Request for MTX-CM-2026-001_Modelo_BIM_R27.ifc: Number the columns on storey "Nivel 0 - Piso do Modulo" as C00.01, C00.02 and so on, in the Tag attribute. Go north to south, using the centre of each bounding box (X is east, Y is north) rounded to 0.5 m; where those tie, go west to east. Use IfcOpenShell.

First a look at what the model holds.

```python
import ifcopenshell
import ifcopenshell.util.element
import ifcopenshell.util.placement

model = ifcopenshell.open("MTX-CM-2026-001_Modelo_BIM_R27.ifc")
print(model.schema)
storey = next(s for s in model.by_type("IfcBuildingStorey") if s.Name == "Nivel 0 - Piso do Modulo")
columns = [e for e in ifcopenshell.util.element.get_decomposition(storey) if e.is_a("IfcColumn")]
for e in sorted(columns, key=lambda e: e.id()):
    origin = ifcopenshell.util.placement.get_local_placement(e.ObjectPlacement)[:3, 3]
    print(e.id(), e.Tag, e.Name, origin.round(2) + 0.0, sep=" | ")
```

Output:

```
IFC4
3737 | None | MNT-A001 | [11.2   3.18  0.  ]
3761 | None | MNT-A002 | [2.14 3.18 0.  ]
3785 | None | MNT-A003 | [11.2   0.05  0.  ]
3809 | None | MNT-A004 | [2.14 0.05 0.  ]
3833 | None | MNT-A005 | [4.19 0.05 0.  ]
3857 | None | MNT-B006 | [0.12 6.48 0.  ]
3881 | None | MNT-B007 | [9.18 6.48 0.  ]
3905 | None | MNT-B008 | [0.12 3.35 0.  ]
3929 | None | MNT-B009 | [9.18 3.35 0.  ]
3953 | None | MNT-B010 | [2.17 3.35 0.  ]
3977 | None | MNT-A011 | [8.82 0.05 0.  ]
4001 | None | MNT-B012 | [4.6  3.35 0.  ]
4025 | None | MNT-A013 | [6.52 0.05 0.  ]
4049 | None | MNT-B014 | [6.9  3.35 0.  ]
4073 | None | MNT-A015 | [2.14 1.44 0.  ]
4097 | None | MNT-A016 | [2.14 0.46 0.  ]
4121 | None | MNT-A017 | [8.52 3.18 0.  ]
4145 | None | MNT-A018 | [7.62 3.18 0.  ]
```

```python
import ifcopenshell
import ifcopenshell.geom
import ifcopenshell.util.element
import ifcopenshell.util.shape

model = ifcopenshell.open("MTX-CM-2026-001_Modelo_BIM_R27.ifc")
settings = ifcopenshell.geom.settings()
settings.set("use-world-coords", True)


def centre(element):
    shape = ifcopenshell.geom.create_shape(settings, element)
    return ifcopenshell.util.shape.get_bbox_centroid(shape.geometry)


storey = next(s for s in model.by_type("IfcBuildingStorey") if s.Name == "Nivel 0 - Piso do Modulo")
columns = [e for e in ifcopenshell.util.element.get_decomposition(storey) if e.is_a("IfcColumn")]

# Insertion points can sit at a corner or the storey origin, so sort by the geometry (in metres).
centres = {e: centre(e) for e in columns}
columns.sort(key=lambda e: (-round(centres[e][1] / 0.5), centres[e][0]))

for i, e in enumerate(columns, start=1):
    number = f"C00.{i:02d}"
    e.Tag = number
    print(e.id(), number)

model.write("MTX-CM-2026-001_Modelo_BIM_R27-out.ifc")
```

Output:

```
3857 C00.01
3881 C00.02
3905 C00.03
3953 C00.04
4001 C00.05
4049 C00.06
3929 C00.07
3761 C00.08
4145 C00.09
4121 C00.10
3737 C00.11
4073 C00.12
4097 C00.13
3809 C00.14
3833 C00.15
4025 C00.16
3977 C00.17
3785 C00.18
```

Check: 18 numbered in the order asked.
